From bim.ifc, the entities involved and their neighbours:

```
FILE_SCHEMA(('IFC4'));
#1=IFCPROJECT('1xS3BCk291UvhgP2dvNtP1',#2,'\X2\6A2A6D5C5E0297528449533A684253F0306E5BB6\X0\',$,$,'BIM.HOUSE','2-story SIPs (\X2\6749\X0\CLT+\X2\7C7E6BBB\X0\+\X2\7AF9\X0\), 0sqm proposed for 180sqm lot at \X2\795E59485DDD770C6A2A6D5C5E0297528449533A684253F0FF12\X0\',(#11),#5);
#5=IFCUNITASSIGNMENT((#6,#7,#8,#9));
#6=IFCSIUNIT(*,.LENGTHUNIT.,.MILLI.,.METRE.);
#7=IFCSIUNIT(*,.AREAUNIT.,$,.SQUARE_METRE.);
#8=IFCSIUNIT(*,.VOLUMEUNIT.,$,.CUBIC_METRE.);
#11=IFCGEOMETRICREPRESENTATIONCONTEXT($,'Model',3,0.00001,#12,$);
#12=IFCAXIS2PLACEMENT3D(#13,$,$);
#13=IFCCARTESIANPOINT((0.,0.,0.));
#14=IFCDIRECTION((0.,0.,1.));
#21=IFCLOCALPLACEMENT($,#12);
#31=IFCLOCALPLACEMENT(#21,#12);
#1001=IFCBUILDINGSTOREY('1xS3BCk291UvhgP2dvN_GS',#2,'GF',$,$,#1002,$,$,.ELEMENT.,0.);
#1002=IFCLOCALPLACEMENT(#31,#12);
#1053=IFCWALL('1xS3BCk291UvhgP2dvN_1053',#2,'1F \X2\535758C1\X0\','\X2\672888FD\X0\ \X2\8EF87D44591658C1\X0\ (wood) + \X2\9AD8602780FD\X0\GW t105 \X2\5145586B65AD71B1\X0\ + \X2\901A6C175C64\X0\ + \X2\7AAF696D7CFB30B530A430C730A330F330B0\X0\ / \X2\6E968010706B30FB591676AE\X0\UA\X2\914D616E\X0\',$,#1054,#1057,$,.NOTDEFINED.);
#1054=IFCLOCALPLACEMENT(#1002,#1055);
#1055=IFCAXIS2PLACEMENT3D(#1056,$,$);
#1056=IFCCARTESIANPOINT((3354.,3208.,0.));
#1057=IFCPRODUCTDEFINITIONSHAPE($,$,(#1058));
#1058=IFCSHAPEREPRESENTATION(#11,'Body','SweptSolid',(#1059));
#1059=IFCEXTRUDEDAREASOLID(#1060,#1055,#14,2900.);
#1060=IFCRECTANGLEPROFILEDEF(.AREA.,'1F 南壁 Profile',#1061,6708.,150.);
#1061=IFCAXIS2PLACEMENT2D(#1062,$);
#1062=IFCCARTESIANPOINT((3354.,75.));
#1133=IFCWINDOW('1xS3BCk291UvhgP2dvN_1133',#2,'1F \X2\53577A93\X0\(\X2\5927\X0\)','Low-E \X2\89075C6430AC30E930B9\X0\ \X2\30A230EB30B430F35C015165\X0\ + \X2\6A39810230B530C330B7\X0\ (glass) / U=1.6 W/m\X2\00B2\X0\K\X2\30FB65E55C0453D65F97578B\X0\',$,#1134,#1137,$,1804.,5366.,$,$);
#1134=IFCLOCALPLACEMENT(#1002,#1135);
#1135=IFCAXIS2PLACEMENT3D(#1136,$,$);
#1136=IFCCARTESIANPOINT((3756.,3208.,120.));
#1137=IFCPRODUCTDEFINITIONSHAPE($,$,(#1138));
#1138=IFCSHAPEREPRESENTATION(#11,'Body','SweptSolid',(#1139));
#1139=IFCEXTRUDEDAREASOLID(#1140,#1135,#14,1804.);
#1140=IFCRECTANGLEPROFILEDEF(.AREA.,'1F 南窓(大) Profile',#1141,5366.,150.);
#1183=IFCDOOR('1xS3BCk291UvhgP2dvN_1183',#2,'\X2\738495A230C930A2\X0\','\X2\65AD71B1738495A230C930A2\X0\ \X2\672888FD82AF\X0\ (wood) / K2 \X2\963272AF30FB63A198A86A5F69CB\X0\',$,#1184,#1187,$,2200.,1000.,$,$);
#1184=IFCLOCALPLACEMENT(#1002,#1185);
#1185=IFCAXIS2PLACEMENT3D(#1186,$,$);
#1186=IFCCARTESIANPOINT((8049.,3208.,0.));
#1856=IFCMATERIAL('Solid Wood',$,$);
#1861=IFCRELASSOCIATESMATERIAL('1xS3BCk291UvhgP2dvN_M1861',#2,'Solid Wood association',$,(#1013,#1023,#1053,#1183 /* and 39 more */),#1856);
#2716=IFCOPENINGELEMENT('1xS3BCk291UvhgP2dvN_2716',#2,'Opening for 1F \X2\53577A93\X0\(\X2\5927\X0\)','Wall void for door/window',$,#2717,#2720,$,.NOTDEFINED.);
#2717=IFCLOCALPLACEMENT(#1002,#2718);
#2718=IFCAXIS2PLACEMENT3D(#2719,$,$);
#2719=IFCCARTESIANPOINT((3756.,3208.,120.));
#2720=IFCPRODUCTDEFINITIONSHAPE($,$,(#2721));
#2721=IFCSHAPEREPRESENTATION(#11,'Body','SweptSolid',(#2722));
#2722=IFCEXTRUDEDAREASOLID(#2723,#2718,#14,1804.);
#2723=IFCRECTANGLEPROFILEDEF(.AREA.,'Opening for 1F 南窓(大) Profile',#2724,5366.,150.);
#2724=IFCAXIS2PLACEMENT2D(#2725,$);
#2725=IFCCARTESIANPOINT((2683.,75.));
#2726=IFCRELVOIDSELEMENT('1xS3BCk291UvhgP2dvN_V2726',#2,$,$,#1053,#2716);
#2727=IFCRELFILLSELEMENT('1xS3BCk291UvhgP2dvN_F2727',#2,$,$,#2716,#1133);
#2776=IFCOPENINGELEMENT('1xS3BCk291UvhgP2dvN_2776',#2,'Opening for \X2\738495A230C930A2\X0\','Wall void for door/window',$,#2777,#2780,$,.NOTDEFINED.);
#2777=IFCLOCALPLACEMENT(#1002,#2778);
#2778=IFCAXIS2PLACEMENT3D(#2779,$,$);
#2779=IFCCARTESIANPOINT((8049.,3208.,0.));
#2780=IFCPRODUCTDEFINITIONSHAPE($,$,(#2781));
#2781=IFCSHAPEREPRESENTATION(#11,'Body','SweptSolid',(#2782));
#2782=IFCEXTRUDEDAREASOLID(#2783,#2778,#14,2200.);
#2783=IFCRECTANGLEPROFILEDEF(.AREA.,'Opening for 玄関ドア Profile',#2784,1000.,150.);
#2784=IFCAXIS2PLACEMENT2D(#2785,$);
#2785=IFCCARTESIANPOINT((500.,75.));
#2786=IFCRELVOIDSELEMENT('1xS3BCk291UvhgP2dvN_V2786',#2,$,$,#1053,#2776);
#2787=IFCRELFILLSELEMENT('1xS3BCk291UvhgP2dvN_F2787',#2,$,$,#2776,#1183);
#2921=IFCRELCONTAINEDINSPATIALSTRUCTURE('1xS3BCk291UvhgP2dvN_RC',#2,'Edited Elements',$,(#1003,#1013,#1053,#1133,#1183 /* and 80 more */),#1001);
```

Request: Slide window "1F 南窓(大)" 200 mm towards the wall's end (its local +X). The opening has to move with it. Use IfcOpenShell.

```python
import ifcopenshell
import ifcopenshell.api.geometry
import ifcopenshell.util.placement
import ifcopenshell.util.unit

model = ifcopenshell.open("bim.ifc")
unit_scale = ifcopenshell.util.unit.calculate_unit_scale(model)

window = model.by_id(1133)
opening = window.FillsVoids[0].RelatingOpeningElement
wall = opening.VoidsElements[0].RelatingBuildingElement

wall_matrix = ifcopenshell.util.placement.get_local_placement(wall.ObjectPlacement)
shift = wall_matrix[:3, 0] * 0.2 / unit_scale
before = ifcopenshell.util.placement.get_local_placement(window.ObjectPlacement)[:3, 3].copy()

# The window is not placed relative to its opening, so move both.
for product in (opening, window):
    matrix = ifcopenshell.util.placement.get_local_placement(product.ObjectPlacement)
    matrix[:3, 3] += shift
    ifcopenshell.api.geometry.edit_object_placement(model, product=product, matrix=matrix, is_si=False)

after = ifcopenshell.util.placement.get_local_placement(window.ObjectPlacement)[:3, 3]
print("window moved by", (after - before).round(3) + 0.0)

model.write("bim_rev.ifc")
```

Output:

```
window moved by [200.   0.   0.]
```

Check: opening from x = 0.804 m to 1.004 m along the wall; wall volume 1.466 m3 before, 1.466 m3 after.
